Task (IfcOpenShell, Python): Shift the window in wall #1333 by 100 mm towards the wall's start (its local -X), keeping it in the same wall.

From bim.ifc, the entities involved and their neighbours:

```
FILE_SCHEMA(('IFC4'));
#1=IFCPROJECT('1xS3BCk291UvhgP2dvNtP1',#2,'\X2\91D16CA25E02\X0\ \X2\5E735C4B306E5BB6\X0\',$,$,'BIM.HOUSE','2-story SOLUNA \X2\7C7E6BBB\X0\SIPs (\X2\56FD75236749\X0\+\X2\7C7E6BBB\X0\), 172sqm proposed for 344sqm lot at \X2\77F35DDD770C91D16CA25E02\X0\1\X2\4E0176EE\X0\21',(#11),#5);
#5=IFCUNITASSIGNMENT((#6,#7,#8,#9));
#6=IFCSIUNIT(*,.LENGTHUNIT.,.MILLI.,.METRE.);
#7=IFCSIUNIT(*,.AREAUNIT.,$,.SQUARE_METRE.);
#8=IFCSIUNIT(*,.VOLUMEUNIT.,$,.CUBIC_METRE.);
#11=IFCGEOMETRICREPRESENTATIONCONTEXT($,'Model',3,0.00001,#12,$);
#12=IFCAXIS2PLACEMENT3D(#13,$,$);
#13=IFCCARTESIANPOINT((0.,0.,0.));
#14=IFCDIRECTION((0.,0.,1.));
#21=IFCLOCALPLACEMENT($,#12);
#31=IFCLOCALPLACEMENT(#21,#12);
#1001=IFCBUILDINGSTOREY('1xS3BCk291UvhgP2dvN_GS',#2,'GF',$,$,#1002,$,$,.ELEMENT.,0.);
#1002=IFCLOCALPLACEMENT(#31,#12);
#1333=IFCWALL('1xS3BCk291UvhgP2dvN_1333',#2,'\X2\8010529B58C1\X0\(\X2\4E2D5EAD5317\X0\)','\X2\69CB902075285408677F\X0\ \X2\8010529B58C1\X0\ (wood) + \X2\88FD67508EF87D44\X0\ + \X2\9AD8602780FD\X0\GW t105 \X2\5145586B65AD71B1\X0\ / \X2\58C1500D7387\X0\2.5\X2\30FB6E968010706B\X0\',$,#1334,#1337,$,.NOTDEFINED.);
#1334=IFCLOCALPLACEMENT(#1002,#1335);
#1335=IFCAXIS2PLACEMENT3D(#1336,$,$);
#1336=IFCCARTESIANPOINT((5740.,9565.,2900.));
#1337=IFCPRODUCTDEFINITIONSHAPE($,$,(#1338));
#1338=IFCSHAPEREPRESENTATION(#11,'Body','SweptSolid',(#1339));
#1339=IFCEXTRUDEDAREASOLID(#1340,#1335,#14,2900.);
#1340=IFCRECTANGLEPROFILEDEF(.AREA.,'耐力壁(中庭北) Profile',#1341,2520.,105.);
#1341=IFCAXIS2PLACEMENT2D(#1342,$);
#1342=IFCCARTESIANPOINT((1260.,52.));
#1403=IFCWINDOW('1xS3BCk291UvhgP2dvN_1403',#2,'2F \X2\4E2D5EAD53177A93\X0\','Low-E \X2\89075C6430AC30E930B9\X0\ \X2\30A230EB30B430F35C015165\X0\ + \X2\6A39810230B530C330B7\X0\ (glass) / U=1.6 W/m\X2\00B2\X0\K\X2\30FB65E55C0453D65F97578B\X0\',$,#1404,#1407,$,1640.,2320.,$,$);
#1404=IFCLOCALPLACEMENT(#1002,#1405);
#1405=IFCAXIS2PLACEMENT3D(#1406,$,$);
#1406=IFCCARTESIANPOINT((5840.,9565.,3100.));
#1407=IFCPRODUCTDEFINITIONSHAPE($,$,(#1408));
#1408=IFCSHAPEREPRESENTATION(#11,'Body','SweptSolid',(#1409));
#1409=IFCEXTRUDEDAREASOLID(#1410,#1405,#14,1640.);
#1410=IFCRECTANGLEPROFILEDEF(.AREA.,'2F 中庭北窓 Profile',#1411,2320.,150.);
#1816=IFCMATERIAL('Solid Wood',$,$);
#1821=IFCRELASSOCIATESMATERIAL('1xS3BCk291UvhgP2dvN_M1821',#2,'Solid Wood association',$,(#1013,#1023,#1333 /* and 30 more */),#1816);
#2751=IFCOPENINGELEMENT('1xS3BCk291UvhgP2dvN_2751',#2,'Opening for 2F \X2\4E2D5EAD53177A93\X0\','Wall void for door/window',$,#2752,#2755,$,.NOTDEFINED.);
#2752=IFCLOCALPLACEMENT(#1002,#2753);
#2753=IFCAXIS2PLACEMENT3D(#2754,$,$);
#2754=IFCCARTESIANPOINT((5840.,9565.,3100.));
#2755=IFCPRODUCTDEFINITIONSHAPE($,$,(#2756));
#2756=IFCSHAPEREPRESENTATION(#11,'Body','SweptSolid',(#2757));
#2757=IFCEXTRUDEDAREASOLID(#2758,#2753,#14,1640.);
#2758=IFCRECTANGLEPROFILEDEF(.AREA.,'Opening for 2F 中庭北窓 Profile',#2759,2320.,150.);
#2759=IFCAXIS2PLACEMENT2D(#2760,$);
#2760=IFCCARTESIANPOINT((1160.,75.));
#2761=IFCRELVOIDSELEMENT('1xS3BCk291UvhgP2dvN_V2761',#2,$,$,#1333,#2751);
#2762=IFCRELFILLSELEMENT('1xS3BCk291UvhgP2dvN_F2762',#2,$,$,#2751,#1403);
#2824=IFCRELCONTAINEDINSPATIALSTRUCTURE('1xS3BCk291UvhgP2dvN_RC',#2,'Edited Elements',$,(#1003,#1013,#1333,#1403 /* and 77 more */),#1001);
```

```python
import ifcopenshell
import ifcopenshell.api.geometry
import ifcopenshell.util.placement
import ifcopenshell.util.unit

model = ifcopenshell.open("bim.ifc")
unit_scale = ifcopenshell.util.unit.calculate_unit_scale(model)

window = model.by_guid("1xS3BCk291UvhgP2dvN_1403")
opening = window.FillsVoids[0].RelatingOpeningElement
wall = opening.VoidsElements[0].RelatingBuildingElement

wall_matrix = ifcopenshell.util.placement.get_local_placement(wall.ObjectPlacement)
shift = wall_matrix[:3, 0] * -0.1 / unit_scale
before = ifcopenshell.util.placement.get_local_placement(window.ObjectPlacement)[:3, 3].copy()

# The window is not placed relative to its opening, so move both.
for product in (opening, window):
    matrix = ifcopenshell.util.placement.get_local_placement(product.ObjectPlacement)
    matrix[:3, 3] += shift
    ifcopenshell.api.geometry.edit_object_placement(model, product=product, matrix=matrix, is_si=False)

after = ifcopenshell.util.placement.get_local_placement(window.ObjectPlacement)[:3, 3]
print("window moved by", (after - before).round(3) + 0.0)

model.write("bim_rev.ifc")
```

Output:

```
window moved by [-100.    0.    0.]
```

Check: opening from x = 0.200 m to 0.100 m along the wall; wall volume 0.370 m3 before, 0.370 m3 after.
